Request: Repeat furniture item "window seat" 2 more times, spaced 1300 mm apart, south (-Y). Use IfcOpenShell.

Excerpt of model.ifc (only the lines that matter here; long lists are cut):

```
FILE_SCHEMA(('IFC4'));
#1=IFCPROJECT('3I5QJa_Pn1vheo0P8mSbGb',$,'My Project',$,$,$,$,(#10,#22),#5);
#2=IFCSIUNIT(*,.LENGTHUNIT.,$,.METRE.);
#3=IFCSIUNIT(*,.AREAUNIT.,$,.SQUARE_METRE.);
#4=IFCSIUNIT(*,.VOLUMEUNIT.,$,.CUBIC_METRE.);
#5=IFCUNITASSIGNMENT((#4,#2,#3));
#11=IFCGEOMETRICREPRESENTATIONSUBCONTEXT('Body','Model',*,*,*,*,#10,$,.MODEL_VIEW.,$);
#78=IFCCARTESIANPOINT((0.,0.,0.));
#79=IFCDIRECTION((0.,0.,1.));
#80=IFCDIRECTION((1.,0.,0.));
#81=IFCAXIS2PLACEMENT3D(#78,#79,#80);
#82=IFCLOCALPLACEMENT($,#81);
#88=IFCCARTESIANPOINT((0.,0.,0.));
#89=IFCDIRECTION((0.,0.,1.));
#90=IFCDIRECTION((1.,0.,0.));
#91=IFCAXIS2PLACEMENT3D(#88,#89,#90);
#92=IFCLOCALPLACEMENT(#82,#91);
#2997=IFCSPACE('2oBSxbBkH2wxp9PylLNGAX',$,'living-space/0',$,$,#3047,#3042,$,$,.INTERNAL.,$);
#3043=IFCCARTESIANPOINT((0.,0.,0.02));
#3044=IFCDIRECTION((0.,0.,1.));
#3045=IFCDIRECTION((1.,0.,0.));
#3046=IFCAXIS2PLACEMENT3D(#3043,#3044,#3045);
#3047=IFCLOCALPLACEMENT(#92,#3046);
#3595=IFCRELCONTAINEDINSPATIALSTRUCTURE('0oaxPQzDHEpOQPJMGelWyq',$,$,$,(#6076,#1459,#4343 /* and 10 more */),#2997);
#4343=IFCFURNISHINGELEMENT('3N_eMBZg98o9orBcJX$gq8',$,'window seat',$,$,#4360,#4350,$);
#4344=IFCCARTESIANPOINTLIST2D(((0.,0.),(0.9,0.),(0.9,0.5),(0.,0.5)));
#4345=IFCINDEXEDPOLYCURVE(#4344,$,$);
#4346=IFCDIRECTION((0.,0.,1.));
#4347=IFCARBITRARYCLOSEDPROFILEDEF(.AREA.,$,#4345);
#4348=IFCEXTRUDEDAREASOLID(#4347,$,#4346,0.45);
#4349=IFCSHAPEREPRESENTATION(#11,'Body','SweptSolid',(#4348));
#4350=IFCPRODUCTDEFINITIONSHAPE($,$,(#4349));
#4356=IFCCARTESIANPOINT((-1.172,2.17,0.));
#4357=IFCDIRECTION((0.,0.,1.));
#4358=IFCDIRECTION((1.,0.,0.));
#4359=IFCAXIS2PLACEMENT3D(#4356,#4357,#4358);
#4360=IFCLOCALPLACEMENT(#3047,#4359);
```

```python
import numpy as np
import ifcopenshell
import ifcopenshell.api.geometry
import ifcopenshell.api.root
import ifcopenshell.util.element
import ifcopenshell.util.placement

model = ifcopenshell.open("model.ifc")

source = model.by_guid("3N_eMBZg98o9orBcJX$gq8")
base = ifcopenshell.util.placement.get_local_placement(source.ObjectPlacement)
step = np.array([0.0, -1.0, 0.0]) * 1.3

for i in range(1, 3):
    copy = ifcopenshell.api.root.copy_class(model, product=source)
    copy.Representation = ifcopenshell.util.element.copy_deep(
        model, source.Representation, exclude=["IfcGeometricRepresentationContext", "IfcRepresentationMap"]
    )
    matrix = base.copy()
    matrix[:3, 3] += i * step
    print("added at", matrix[:3, 3].round(3) + 0.0)
    ifcopenshell.api.geometry.edit_object_placement(model, product=copy, matrix=matrix, is_si=False)

model.write("model_edited.ifc")
```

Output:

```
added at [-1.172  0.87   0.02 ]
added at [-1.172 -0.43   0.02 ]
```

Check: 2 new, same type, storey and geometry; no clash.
